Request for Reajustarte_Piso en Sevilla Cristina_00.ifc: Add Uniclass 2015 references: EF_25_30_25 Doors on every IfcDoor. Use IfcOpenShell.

First a look at what the model holds.

```python
import ifcopenshell

model = ifcopenshell.open("Reajustarte_Piso en Sevilla Cristina_00.ifc")
print(model.schema)
print("classifications:", [c.Name for c in model.by_type("IfcClassification")])
for ifc_class in ("IfcDoor", "IfcRoof", "IfcStair", "IfcWall", "IfcWindow"):
    print(ifc_class, len(model.by_type(ifc_class)))
```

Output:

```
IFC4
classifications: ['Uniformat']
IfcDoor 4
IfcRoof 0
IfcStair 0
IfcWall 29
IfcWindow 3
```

```python
import ifcopenshell
import ifcopenshell.api.classification

model = ifcopenshell.open("Reajustarte_Piso en Sevilla Cristina_00.ifc")

system = ifcopenshell.api.classification.add_classification(model, classification="Uniclass 2015")

codes = {
    "IfcDoor": ("EF_25_30_25", "Doors"),
}
for ifc_class, (code, name) in codes.items():
    products = model.by_type(ifc_class)
    ifcopenshell.api.classification.add_reference(
        model, products=products, classification=system, identification=code, name=name
    )
    print(code, len(products))

model.write("Reajustarte_Piso en Sevilla Cristina_00_updated.ifc")
```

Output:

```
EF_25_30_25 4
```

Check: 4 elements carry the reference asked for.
